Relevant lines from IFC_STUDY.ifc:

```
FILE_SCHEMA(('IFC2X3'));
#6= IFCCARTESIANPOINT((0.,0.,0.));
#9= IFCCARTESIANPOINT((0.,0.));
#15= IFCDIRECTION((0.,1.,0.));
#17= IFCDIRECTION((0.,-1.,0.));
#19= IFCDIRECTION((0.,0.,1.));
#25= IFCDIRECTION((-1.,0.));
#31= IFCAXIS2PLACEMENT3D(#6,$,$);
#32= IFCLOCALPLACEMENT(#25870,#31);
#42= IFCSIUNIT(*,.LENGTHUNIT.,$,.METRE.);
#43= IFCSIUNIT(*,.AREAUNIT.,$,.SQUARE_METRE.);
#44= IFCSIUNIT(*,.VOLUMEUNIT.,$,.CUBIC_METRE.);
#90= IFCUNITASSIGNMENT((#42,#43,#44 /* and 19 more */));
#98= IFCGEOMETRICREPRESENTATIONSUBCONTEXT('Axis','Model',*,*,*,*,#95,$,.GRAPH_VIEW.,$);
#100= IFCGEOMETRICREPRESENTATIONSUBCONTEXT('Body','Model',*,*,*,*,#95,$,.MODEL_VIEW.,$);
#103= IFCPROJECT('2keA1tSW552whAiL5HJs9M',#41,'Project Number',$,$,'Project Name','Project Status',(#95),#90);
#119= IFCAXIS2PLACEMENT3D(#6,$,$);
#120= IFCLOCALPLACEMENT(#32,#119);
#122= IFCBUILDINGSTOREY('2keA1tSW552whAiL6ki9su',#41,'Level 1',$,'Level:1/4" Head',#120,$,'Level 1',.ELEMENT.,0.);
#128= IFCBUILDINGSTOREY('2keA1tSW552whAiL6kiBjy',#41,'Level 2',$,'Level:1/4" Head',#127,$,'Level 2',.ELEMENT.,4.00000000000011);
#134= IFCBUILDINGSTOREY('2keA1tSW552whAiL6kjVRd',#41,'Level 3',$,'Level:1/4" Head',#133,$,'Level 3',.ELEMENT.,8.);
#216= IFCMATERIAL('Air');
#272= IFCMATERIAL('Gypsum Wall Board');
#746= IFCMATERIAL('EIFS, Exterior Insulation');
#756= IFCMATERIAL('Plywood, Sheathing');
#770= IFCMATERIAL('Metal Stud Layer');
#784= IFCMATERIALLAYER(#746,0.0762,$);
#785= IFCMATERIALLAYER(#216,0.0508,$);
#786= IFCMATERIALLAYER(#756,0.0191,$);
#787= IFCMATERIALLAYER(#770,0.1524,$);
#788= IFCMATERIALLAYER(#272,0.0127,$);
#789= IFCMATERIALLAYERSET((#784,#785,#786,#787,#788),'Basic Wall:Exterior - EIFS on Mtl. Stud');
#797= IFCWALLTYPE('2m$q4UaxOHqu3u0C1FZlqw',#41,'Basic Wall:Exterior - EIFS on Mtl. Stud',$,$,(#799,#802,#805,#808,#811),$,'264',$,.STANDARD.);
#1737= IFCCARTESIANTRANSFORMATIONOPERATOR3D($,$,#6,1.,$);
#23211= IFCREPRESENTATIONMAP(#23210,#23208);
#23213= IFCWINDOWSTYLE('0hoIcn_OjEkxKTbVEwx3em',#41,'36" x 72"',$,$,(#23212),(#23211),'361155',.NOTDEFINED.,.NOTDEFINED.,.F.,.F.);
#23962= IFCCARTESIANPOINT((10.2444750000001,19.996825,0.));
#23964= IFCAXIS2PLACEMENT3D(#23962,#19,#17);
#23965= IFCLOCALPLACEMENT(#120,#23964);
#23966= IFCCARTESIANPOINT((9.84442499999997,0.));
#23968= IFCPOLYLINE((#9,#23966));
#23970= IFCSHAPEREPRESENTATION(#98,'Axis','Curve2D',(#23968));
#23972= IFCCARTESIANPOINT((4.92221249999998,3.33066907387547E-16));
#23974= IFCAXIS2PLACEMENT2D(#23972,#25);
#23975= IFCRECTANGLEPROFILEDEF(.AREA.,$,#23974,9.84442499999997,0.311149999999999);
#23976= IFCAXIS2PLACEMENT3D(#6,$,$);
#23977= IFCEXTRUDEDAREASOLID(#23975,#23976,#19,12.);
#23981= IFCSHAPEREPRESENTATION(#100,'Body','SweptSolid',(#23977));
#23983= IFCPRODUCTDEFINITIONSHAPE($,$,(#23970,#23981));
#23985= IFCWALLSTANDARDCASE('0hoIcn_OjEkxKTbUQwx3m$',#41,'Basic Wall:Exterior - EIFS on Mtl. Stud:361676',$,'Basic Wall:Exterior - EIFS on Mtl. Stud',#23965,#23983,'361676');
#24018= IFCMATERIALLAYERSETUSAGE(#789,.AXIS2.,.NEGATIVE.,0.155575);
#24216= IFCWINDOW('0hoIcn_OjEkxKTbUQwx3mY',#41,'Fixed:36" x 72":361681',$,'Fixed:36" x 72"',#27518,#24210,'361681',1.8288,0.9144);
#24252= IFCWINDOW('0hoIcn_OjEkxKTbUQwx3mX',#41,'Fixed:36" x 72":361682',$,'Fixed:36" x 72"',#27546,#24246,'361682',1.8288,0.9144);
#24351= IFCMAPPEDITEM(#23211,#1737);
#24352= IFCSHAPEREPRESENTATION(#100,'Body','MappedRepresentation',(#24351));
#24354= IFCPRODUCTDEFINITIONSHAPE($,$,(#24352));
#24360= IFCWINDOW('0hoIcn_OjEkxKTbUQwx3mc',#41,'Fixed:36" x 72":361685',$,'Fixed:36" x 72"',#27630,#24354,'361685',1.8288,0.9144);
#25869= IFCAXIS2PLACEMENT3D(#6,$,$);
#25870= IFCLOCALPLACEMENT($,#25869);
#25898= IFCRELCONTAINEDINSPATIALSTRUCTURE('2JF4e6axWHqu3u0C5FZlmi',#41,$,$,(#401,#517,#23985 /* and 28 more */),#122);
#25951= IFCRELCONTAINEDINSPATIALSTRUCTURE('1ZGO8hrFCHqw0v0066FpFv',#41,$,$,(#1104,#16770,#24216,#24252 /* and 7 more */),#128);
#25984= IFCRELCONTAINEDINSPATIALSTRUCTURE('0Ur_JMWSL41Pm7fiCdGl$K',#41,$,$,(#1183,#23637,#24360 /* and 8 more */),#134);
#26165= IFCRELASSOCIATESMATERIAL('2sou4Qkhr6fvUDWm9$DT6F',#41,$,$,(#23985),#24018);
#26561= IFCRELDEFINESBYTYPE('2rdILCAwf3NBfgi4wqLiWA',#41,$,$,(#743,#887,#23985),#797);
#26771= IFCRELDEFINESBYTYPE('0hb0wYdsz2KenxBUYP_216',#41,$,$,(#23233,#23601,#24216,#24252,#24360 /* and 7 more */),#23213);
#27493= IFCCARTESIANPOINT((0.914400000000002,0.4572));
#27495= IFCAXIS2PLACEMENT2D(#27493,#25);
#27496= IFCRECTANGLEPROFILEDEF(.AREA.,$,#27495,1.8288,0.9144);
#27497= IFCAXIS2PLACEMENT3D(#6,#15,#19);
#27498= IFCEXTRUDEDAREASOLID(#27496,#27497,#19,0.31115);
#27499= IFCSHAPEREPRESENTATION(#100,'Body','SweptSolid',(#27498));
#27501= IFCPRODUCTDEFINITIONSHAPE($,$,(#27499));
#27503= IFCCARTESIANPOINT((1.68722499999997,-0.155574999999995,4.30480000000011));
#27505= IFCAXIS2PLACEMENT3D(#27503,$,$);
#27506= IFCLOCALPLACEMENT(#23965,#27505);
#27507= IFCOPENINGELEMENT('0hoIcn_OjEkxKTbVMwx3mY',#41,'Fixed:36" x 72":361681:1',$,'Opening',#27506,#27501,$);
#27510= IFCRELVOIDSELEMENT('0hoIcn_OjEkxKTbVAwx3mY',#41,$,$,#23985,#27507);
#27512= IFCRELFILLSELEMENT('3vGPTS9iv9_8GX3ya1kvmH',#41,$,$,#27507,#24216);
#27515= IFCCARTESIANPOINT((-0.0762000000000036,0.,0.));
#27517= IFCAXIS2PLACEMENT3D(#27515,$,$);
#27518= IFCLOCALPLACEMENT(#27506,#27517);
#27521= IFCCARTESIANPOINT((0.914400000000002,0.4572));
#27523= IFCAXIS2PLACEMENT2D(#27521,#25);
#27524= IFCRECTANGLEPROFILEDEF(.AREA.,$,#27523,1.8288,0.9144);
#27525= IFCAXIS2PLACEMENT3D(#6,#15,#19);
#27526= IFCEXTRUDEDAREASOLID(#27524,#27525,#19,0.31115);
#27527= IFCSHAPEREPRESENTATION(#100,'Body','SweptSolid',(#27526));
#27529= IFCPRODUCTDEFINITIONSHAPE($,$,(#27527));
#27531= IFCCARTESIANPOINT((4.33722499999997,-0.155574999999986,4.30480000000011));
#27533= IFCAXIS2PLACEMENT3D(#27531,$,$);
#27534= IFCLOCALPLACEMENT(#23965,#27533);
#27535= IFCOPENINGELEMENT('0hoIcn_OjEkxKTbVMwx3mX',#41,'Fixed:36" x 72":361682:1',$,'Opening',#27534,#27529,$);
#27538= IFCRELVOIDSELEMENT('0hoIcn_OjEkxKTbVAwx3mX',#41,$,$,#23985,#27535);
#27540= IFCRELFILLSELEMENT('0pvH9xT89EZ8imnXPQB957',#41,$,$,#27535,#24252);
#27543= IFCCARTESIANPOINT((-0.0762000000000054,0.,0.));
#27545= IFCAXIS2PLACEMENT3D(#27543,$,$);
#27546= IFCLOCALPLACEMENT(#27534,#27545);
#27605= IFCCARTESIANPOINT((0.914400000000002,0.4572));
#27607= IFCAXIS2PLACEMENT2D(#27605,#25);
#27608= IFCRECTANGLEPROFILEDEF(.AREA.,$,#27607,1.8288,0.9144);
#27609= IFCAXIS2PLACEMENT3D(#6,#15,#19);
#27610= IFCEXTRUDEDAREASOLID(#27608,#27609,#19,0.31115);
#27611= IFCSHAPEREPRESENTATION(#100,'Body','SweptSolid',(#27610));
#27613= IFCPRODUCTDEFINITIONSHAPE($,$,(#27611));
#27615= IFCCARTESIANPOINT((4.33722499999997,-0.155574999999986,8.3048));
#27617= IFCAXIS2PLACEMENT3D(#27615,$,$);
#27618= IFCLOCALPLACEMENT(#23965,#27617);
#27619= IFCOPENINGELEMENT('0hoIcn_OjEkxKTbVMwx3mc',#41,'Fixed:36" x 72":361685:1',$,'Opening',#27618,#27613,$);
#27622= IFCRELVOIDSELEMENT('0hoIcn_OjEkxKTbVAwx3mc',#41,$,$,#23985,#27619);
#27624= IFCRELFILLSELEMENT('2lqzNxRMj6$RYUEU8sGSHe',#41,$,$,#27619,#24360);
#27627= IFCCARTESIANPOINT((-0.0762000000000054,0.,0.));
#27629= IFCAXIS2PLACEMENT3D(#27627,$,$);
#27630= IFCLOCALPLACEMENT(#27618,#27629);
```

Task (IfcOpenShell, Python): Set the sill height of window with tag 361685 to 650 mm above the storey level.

```python
import numpy as np
import ifcopenshell
import ifcopenshell.api.geometry
import ifcopenshell.geom
import ifcopenshell.util.element
import ifcopenshell.util.placement
import ifcopenshell.util.shape
import ifcopenshell.util.unit

model = ifcopenshell.open("IFC_STUDY.ifc")
unit_scale = ifcopenshell.util.unit.calculate_unit_scale(model)

window = model.by_guid("0hoIcn_OjEkxKTbUQwx3mc")
opening = window.FillsVoids[0].RelatingOpeningElement
storey = ifcopenshell.util.element.get_container(window, ifc_class="IfcBuildingStorey")
level = ifcopenshell.util.placement.get_local_placement(storey.ObjectPlacement)[2, 3]

# The opening's origin need not be at the sill, so measure its lowest point.
shape = ifcopenshell.geom.create_shape(ifcopenshell.geom.settings(), opening)
bottom = ifcopenshell.util.shape.get_shape_bottom_elevation(shape, shape.geometry) / unit_scale
dz = level + 0.65 / unit_scale - bottom

shift = np.array([0.0, 0.0, dz])
# The window is placed relative to its opening, so it follows when the opening moves.
matrix = ifcopenshell.util.placement.get_local_placement(opening.ObjectPlacement)
matrix[:3, 3] += shift
ifcopenshell.api.geometry.edit_object_placement(
    model, product=opening, matrix=matrix, is_si=False, should_transform_children=True
)

print(f"moved by {dz * unit_scale:+.3f} m")

model.write("IFC_STUDY_edited.ifc")
```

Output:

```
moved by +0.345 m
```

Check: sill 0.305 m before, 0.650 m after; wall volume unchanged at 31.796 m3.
